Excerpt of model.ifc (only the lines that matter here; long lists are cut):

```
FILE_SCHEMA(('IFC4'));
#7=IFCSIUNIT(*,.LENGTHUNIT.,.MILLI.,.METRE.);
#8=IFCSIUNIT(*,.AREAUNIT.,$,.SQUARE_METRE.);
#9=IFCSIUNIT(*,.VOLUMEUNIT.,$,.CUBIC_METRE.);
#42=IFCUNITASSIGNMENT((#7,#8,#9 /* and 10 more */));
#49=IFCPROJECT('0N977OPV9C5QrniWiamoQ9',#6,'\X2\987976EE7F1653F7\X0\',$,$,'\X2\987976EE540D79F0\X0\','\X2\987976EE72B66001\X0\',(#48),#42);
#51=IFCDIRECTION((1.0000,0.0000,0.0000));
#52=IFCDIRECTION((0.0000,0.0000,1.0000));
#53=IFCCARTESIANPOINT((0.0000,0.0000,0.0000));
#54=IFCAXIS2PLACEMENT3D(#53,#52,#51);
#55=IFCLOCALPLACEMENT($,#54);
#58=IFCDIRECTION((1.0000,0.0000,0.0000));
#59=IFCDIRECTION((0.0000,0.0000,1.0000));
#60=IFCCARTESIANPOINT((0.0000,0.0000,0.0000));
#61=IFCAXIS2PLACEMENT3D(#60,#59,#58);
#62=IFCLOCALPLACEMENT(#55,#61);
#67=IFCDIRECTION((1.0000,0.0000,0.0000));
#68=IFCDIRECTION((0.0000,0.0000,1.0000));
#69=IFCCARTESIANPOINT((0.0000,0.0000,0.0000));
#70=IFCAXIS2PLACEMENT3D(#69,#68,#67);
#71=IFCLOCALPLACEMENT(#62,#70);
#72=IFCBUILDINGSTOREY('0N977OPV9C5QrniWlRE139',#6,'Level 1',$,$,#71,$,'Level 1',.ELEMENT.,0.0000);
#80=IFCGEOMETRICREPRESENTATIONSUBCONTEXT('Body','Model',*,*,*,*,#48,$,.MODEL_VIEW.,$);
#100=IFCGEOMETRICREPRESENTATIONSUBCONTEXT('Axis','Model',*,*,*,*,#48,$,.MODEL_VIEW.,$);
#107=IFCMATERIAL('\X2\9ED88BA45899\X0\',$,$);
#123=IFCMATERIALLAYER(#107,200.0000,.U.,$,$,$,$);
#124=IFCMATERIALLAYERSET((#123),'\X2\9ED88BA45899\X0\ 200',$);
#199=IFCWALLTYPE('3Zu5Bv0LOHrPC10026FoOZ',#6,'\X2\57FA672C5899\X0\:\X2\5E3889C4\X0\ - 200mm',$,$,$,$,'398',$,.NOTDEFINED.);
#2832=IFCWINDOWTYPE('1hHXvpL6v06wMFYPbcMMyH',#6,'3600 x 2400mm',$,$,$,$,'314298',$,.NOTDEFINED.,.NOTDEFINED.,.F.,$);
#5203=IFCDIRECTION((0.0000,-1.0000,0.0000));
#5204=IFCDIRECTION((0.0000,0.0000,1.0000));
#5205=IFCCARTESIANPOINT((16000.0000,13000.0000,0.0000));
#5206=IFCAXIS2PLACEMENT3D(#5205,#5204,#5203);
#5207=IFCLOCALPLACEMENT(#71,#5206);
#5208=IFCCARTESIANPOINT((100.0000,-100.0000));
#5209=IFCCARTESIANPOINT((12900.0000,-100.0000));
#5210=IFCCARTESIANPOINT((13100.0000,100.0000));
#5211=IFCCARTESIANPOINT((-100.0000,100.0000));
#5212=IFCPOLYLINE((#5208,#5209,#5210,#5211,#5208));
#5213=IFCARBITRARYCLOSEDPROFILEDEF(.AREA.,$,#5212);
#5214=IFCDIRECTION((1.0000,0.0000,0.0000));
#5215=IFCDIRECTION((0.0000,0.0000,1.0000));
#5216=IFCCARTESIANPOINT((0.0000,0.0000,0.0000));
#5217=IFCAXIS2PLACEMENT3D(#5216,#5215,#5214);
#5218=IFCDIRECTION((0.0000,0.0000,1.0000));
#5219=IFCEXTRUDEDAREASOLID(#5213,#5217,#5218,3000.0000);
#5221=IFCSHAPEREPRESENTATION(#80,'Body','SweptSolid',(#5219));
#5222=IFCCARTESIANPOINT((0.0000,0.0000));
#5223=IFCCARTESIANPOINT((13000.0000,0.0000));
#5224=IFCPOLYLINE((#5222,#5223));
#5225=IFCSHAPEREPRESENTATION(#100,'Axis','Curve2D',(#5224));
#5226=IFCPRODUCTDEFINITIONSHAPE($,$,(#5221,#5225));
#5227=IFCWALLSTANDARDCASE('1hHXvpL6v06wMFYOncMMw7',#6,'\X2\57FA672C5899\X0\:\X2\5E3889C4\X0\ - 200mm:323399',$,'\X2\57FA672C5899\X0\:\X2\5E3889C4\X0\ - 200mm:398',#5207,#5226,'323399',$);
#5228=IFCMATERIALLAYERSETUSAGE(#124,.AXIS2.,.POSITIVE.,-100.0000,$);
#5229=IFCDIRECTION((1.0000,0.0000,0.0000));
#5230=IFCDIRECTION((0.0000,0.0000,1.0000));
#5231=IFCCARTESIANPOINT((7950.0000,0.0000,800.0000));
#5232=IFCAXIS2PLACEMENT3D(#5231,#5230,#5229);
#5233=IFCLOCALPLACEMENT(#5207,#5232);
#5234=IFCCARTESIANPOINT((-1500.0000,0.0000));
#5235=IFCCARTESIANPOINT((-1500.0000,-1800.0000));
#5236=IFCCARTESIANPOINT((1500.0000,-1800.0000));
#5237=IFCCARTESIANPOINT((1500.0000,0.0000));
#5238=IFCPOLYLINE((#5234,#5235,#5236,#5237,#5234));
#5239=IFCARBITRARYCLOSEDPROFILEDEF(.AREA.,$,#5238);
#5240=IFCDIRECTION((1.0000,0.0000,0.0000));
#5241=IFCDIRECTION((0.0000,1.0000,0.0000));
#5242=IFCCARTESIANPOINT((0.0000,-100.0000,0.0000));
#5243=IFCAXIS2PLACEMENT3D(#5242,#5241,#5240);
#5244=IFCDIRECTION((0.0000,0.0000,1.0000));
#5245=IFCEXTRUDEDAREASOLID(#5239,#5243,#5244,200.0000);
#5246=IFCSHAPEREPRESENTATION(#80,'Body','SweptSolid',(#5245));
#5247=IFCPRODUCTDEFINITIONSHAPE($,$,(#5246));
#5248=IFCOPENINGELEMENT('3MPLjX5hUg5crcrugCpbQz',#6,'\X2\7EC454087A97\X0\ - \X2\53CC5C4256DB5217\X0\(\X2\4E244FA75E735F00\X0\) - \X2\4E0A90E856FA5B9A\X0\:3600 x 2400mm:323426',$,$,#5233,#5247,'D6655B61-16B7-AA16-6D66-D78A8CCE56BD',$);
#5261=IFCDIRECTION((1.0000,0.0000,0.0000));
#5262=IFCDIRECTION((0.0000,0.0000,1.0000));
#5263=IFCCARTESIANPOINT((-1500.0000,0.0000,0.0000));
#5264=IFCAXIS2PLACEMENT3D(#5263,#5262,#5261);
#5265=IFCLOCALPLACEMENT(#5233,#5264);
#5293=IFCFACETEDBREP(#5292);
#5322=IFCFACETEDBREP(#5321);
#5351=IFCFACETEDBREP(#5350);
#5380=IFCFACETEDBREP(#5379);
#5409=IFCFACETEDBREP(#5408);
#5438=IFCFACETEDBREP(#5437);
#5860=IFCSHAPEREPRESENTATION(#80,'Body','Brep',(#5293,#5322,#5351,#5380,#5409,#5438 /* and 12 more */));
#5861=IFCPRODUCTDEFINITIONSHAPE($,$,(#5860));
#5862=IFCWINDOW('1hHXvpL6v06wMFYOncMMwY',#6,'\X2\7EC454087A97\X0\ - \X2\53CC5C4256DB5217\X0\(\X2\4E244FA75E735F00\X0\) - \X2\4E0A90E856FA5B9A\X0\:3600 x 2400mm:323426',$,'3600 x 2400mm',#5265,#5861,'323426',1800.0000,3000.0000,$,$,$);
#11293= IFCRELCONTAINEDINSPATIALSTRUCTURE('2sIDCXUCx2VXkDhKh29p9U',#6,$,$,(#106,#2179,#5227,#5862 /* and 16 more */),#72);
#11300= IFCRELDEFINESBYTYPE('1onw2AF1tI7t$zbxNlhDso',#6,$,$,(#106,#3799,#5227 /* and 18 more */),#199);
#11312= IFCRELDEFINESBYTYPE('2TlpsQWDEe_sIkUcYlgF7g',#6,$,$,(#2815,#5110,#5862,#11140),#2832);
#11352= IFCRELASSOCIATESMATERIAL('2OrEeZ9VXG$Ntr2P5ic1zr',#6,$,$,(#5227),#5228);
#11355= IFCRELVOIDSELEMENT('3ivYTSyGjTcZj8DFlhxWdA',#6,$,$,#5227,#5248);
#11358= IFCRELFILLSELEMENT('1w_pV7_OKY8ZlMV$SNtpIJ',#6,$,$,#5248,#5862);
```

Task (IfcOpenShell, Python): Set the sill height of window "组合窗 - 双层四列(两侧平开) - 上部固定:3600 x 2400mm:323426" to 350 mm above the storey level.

```python
import numpy as np
import ifcopenshell
import ifcopenshell.api.geometry
import ifcopenshell.geom
import ifcopenshell.util.element
import ifcopenshell.util.placement
import ifcopenshell.util.shape
import ifcopenshell.util.unit

model = ifcopenshell.open("model.ifc")
unit_scale = ifcopenshell.util.unit.calculate_unit_scale(model)

window = model.by_guid("1hHXvpL6v06wMFYOncMMwY")
opening = window.FillsVoids[0].RelatingOpeningElement
storey = ifcopenshell.util.element.get_container(window, ifc_class="IfcBuildingStorey")
level = ifcopenshell.util.placement.get_local_placement(storey.ObjectPlacement)[2, 3]

# The opening's origin need not be at the sill, so measure its lowest point.
shape = ifcopenshell.geom.create_shape(ifcopenshell.geom.settings(), opening)
bottom = ifcopenshell.util.shape.get_shape_bottom_elevation(shape, shape.geometry) / unit_scale
dz = level + 0.35 / unit_scale - bottom

shift = np.array([0.0, 0.0, dz])
# The window is placed relative to its opening, so it follows when the opening moves.
matrix = ifcopenshell.util.placement.get_local_placement(opening.ObjectPlacement)
matrix[:3, 3] += shift
ifcopenshell.api.geometry.edit_object_placement(
    model, product=opening, matrix=matrix, is_si=False, should_transform_children=True
)

print(f"moved by {dz * unit_scale:+.3f} m")

model.write("model_updated.ifc")
```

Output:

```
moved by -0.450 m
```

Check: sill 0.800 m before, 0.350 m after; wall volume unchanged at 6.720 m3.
